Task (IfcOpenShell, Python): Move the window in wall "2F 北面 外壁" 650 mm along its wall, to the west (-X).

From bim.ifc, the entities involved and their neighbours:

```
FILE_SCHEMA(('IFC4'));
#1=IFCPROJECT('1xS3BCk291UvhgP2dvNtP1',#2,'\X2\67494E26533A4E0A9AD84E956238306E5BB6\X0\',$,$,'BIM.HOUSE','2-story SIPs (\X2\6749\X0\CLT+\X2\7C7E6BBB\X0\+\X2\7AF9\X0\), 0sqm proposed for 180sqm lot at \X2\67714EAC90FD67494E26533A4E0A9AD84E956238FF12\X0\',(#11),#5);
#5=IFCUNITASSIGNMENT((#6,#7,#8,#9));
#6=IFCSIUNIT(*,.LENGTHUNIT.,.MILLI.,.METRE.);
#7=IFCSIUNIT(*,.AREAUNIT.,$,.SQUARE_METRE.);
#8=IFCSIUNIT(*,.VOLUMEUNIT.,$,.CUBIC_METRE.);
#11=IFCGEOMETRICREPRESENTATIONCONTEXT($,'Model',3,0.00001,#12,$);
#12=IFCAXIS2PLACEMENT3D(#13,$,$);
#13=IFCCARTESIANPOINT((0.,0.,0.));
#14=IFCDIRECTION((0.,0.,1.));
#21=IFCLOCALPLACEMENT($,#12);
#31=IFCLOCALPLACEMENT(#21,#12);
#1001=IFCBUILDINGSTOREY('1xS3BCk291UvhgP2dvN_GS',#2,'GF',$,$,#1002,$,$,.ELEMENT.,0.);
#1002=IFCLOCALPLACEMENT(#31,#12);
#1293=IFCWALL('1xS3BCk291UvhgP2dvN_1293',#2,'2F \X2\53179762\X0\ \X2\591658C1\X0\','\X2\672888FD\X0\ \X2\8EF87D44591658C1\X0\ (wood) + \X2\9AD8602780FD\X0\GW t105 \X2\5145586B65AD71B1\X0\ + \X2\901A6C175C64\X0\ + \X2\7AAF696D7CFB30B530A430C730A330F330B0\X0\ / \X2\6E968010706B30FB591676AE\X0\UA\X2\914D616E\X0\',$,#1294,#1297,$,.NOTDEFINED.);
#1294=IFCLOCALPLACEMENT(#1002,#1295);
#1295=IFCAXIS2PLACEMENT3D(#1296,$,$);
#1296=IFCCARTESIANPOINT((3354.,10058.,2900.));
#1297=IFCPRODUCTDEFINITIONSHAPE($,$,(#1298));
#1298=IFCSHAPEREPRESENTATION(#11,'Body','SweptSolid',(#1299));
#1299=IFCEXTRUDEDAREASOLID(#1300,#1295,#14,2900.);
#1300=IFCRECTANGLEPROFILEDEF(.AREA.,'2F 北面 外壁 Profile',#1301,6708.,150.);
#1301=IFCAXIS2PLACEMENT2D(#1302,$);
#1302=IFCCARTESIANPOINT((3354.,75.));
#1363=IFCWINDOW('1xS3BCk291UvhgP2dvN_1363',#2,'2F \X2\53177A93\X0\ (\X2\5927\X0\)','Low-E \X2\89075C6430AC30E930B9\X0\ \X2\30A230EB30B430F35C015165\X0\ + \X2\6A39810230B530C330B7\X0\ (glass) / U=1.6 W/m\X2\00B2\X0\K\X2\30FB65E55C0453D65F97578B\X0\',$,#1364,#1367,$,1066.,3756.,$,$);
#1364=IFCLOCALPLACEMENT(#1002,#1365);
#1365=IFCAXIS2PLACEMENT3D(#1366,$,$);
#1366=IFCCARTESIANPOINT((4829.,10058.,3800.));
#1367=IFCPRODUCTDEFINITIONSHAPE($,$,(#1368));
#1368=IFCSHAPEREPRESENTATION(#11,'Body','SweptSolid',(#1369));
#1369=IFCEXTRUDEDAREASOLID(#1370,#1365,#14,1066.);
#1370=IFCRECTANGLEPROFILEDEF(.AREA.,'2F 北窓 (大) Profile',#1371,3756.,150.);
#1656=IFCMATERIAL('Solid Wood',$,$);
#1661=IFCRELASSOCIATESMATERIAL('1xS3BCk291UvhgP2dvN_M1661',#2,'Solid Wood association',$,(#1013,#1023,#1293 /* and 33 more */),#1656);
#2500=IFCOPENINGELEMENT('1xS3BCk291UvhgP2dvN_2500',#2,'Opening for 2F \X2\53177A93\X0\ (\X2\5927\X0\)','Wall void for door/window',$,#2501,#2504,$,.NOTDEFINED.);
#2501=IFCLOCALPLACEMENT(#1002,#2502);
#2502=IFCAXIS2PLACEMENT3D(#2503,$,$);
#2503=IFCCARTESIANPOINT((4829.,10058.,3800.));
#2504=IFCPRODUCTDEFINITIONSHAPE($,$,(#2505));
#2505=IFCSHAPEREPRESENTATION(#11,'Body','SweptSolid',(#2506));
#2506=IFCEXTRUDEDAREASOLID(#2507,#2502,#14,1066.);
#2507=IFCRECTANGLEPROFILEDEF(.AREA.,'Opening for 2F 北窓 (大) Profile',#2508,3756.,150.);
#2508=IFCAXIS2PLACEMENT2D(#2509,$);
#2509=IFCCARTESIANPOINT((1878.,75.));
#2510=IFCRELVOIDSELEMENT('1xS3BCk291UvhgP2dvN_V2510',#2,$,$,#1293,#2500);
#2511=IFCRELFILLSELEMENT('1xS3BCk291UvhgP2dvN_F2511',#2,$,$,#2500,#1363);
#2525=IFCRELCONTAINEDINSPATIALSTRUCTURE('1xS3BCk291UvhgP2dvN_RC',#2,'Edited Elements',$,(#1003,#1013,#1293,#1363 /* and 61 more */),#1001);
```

```python
import ifcopenshell
import ifcopenshell.api.geometry
import ifcopenshell.util.placement
import ifcopenshell.util.unit

model = ifcopenshell.open("bim.ifc")
unit_scale = ifcopenshell.util.unit.calculate_unit_scale(model)

window = model.by_guid("1xS3BCk291UvhgP2dvN_1363")
opening = window.FillsVoids[0].RelatingOpeningElement
wall = opening.VoidsElements[0].RelatingBuildingElement

wall_matrix = ifcopenshell.util.placement.get_local_placement(wall.ObjectPlacement)
shift = wall_matrix[:3, 0] * -0.65 / unit_scale
before = ifcopenshell.util.placement.get_local_placement(window.ObjectPlacement)[:3, 3].copy()

# The window is not placed relative to its opening, so move both.
for product in (opening, window):
    matrix = ifcopenshell.util.placement.get_local_placement(product.ObjectPlacement)
    matrix[:3, 3] += shift
    ifcopenshell.api.geometry.edit_object_placement(model, product=product, matrix=matrix, is_si=False)

after = ifcopenshell.util.placement.get_local_placement(window.ObjectPlacement)[:3, 3]
print("window moved by", (after - before).round(3) + 0.0)

model.write("bim_edited.ifc")
```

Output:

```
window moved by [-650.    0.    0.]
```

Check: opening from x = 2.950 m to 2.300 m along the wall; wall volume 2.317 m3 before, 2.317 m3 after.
